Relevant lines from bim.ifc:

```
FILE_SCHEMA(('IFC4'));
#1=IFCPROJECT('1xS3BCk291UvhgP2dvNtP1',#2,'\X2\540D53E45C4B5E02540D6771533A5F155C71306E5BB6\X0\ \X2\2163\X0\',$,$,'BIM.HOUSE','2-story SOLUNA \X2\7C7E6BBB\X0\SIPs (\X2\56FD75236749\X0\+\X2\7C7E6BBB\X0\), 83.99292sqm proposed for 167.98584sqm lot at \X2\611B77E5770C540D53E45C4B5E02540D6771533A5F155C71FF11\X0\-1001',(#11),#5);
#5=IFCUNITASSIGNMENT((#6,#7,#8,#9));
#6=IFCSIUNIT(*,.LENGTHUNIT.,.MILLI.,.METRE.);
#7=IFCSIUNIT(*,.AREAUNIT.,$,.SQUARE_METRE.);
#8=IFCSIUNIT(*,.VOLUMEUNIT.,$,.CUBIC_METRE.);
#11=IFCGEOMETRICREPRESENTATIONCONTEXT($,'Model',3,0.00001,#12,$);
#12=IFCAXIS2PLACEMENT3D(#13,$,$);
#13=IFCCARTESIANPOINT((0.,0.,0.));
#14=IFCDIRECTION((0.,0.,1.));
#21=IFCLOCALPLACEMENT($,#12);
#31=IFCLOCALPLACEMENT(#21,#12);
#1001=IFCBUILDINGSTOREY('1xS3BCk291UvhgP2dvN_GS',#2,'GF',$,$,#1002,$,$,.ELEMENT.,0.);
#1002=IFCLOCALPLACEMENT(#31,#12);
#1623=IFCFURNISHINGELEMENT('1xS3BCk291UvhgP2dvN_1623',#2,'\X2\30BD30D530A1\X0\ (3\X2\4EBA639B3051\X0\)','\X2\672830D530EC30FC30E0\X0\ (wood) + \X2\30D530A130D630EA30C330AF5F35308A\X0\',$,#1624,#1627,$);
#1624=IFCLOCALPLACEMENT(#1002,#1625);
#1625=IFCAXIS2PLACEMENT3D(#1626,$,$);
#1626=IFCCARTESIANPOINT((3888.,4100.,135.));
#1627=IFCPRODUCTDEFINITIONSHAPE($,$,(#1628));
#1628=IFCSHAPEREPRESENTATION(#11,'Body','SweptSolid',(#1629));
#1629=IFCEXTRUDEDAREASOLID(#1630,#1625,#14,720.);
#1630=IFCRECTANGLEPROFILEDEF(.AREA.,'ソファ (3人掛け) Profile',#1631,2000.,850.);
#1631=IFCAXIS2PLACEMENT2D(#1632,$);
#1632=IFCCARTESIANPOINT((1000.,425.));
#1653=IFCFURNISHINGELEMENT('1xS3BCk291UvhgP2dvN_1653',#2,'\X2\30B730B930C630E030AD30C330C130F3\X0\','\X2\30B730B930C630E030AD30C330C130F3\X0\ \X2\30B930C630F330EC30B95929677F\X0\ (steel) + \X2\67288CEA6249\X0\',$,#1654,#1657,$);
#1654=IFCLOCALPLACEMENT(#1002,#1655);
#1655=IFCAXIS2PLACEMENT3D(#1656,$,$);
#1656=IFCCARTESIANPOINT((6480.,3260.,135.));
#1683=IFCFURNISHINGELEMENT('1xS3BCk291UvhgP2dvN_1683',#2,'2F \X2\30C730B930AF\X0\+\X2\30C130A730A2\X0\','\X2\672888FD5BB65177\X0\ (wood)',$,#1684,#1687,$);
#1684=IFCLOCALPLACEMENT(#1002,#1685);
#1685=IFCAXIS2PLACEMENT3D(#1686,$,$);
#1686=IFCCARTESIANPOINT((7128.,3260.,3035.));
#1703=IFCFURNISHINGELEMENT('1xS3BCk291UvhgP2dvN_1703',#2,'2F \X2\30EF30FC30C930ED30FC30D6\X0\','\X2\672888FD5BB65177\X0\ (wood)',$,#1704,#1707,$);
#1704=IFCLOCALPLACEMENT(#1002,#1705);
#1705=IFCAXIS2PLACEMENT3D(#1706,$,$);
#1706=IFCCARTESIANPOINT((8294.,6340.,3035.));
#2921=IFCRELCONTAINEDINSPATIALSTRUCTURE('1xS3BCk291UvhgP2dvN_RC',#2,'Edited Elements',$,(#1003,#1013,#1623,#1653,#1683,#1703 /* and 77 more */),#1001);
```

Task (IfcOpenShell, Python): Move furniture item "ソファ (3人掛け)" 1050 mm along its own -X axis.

```python
import ifcopenshell
import ifcopenshell.api.geometry
import ifcopenshell.util.placement

model = ifcopenshell.open("bim.ifc")

item = model.by_id(1623)
matrix = ifcopenshell.util.placement.get_local_placement(item.ObjectPlacement)
matrix[:3, 3] -= matrix[:3, 0] * 1050.0
ifcopenshell.api.geometry.edit_object_placement(model, product=item, matrix=matrix, is_si=False)

print(ifcopenshell.util.placement.get_local_placement(item.ObjectPlacement).round(3) + 0.0)

model.write("bim_updated.ifc")
```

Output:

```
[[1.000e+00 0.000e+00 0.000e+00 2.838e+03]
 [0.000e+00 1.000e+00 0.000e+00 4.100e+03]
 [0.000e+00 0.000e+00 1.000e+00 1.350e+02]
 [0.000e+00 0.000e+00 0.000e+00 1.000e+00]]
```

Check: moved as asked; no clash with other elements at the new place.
